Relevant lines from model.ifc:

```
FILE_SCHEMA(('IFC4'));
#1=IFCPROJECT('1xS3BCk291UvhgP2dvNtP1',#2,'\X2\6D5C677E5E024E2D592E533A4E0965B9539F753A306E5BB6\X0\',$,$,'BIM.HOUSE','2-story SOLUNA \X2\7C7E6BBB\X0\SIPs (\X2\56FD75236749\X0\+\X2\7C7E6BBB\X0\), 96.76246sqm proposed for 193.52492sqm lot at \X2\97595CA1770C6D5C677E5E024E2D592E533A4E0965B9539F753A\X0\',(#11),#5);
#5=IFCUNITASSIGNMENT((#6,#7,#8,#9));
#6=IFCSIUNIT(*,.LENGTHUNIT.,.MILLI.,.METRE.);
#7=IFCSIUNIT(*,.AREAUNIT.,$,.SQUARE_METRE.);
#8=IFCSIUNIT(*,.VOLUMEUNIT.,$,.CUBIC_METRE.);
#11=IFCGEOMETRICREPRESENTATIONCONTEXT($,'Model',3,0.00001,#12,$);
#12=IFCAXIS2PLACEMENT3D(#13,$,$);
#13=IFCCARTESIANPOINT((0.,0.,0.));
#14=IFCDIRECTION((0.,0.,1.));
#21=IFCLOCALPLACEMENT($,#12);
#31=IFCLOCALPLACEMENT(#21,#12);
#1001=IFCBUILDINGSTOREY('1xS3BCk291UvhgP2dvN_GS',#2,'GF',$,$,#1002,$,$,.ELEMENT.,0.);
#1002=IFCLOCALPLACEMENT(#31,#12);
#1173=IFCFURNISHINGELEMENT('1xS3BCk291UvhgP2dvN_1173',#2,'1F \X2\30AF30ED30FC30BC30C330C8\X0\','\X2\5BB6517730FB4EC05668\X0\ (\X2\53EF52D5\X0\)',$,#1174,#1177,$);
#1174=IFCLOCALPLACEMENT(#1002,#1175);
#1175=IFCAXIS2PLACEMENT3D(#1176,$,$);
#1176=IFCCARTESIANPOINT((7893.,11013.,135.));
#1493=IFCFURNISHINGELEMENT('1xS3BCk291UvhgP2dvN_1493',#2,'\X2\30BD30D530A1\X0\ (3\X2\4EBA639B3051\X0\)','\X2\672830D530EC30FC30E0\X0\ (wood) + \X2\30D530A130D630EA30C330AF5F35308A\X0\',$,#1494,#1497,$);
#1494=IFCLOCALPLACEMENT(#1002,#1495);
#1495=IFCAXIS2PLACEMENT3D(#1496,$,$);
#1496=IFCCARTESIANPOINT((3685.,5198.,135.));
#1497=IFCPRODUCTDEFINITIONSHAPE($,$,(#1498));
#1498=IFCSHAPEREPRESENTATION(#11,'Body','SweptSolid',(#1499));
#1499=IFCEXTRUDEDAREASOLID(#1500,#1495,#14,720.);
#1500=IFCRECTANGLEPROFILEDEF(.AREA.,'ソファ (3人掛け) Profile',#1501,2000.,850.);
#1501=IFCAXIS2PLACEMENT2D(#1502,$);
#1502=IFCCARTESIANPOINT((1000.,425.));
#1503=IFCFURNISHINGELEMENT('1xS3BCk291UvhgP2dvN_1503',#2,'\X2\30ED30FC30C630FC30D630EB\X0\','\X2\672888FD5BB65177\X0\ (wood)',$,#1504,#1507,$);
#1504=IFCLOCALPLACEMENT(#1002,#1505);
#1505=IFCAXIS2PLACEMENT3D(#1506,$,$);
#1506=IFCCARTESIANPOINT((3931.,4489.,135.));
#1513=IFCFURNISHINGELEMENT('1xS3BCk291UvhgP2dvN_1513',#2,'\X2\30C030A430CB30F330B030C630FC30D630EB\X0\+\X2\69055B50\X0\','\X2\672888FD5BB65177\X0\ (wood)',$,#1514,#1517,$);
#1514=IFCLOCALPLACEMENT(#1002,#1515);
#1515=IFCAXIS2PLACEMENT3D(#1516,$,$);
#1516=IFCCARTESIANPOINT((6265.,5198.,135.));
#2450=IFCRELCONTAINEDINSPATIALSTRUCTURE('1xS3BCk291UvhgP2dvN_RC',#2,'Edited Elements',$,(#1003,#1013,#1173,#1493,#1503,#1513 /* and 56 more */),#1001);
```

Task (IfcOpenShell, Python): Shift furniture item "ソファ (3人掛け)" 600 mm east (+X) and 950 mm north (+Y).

```python
import ifcopenshell
import ifcopenshell.api.geometry
import ifcopenshell.util.placement
import ifcopenshell.util.unit

model = ifcopenshell.open("model.ifc")
unit_scale = ifcopenshell.util.unit.calculate_unit_scale(model)

item = model.by_guid("1xS3BCk291UvhgP2dvN_1493")
matrix = ifcopenshell.util.placement.get_local_placement(item.ObjectPlacement)
matrix[0, 3] += 0.6 / unit_scale
matrix[1, 3] += 0.95 / unit_scale
ifcopenshell.api.geometry.edit_object_placement(model, product=item, matrix=matrix, is_si=False)

print(ifcopenshell.util.placement.get_local_placement(item.ObjectPlacement).round(3) + 0.0)

model.write("model_v2.ifc")
```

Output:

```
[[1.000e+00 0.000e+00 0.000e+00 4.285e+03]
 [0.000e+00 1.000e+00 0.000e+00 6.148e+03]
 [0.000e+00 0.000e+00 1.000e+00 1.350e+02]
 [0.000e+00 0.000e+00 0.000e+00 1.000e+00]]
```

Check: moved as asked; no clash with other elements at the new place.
